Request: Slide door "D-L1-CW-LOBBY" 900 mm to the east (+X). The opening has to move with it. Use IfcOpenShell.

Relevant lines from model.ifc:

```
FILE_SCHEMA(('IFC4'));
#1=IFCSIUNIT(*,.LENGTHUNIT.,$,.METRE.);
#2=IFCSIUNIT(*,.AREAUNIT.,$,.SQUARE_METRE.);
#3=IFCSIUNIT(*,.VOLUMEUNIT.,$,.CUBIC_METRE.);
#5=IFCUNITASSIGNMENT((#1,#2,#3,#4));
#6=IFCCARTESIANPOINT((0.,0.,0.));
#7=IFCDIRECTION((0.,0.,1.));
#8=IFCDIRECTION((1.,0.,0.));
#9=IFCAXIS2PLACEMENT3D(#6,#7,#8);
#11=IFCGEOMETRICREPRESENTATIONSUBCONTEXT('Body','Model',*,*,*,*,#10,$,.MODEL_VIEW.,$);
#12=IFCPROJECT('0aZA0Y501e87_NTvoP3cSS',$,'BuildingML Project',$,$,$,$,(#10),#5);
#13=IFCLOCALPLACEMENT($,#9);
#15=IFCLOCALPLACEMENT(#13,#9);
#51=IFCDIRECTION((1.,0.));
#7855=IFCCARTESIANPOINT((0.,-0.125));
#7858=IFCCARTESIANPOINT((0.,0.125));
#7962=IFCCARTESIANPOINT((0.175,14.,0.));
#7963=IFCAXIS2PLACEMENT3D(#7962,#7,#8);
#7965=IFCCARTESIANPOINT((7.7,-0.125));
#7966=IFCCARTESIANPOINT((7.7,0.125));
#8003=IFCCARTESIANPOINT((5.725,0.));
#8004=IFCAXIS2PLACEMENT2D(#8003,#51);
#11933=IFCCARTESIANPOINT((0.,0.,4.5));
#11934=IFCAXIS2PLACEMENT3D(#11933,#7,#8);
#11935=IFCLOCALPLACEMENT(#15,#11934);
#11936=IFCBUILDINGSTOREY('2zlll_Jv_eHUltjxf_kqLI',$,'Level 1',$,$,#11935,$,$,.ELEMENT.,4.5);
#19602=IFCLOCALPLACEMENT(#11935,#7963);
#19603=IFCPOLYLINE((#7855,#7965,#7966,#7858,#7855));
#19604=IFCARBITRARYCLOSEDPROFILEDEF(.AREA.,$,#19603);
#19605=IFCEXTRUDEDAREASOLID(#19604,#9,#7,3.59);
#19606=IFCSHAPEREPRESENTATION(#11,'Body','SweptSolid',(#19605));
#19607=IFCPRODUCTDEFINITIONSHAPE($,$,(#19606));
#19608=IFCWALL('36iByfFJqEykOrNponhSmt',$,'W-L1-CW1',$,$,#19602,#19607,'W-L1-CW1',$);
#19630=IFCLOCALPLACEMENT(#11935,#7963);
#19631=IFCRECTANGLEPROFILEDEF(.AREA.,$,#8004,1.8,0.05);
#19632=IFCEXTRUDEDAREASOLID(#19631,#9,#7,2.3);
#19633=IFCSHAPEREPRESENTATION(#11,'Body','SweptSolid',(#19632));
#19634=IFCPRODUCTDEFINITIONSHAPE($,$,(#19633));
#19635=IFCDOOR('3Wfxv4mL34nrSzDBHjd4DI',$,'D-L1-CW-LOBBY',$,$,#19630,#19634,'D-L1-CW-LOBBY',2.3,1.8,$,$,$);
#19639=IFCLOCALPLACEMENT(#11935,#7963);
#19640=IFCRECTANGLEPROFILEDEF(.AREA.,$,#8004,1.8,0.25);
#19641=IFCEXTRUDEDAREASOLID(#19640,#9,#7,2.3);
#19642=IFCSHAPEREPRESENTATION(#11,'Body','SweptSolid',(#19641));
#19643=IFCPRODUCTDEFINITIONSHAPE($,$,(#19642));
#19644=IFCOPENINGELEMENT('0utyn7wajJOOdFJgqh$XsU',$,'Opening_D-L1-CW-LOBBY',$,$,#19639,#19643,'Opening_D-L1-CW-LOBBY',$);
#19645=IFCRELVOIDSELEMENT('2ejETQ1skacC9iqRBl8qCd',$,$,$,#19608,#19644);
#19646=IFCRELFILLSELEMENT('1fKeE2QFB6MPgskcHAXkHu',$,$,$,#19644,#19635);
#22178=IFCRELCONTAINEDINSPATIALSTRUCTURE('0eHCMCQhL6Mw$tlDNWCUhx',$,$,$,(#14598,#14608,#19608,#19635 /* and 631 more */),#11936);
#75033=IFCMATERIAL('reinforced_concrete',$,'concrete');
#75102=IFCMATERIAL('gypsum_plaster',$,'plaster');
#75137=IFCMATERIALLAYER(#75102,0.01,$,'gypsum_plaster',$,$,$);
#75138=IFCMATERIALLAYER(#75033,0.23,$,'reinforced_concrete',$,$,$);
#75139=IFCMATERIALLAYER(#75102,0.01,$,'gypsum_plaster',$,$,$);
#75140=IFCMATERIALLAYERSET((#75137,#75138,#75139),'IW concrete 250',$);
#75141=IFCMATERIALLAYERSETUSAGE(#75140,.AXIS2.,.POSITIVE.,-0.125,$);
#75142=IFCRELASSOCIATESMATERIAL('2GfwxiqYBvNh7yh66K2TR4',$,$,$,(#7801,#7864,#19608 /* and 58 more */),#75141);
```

```python
import ifcopenshell
import ifcopenshell.api.geometry
import ifcopenshell.util.placement

model = ifcopenshell.open("model.ifc")

door = model.by_id(19635)
opening = door.FillsVoids[0].RelatingOpeningElement
wall = opening.VoidsElements[0].RelatingBuildingElement

wall_matrix = ifcopenshell.util.placement.get_local_placement(wall.ObjectPlacement)
shift = wall_matrix[:3, 0] * 0.9
before = ifcopenshell.util.placement.get_local_placement(door.ObjectPlacement)[:3, 3].copy()

# The door is not placed relative to its opening, so move both.
for product in (opening, door):
    matrix = ifcopenshell.util.placement.get_local_placement(product.ObjectPlacement)
    matrix[:3, 3] += shift
    ifcopenshell.api.geometry.edit_object_placement(model, product=product, matrix=matrix, is_si=False)

after = ifcopenshell.util.placement.get_local_placement(door.ObjectPlacement)[:3, 3]
print("door moved by", (after - before).round(3) + 0.0)

model.write("model-out.ifc")
```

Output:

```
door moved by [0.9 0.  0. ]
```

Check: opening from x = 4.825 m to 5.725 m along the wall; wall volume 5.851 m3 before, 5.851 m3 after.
